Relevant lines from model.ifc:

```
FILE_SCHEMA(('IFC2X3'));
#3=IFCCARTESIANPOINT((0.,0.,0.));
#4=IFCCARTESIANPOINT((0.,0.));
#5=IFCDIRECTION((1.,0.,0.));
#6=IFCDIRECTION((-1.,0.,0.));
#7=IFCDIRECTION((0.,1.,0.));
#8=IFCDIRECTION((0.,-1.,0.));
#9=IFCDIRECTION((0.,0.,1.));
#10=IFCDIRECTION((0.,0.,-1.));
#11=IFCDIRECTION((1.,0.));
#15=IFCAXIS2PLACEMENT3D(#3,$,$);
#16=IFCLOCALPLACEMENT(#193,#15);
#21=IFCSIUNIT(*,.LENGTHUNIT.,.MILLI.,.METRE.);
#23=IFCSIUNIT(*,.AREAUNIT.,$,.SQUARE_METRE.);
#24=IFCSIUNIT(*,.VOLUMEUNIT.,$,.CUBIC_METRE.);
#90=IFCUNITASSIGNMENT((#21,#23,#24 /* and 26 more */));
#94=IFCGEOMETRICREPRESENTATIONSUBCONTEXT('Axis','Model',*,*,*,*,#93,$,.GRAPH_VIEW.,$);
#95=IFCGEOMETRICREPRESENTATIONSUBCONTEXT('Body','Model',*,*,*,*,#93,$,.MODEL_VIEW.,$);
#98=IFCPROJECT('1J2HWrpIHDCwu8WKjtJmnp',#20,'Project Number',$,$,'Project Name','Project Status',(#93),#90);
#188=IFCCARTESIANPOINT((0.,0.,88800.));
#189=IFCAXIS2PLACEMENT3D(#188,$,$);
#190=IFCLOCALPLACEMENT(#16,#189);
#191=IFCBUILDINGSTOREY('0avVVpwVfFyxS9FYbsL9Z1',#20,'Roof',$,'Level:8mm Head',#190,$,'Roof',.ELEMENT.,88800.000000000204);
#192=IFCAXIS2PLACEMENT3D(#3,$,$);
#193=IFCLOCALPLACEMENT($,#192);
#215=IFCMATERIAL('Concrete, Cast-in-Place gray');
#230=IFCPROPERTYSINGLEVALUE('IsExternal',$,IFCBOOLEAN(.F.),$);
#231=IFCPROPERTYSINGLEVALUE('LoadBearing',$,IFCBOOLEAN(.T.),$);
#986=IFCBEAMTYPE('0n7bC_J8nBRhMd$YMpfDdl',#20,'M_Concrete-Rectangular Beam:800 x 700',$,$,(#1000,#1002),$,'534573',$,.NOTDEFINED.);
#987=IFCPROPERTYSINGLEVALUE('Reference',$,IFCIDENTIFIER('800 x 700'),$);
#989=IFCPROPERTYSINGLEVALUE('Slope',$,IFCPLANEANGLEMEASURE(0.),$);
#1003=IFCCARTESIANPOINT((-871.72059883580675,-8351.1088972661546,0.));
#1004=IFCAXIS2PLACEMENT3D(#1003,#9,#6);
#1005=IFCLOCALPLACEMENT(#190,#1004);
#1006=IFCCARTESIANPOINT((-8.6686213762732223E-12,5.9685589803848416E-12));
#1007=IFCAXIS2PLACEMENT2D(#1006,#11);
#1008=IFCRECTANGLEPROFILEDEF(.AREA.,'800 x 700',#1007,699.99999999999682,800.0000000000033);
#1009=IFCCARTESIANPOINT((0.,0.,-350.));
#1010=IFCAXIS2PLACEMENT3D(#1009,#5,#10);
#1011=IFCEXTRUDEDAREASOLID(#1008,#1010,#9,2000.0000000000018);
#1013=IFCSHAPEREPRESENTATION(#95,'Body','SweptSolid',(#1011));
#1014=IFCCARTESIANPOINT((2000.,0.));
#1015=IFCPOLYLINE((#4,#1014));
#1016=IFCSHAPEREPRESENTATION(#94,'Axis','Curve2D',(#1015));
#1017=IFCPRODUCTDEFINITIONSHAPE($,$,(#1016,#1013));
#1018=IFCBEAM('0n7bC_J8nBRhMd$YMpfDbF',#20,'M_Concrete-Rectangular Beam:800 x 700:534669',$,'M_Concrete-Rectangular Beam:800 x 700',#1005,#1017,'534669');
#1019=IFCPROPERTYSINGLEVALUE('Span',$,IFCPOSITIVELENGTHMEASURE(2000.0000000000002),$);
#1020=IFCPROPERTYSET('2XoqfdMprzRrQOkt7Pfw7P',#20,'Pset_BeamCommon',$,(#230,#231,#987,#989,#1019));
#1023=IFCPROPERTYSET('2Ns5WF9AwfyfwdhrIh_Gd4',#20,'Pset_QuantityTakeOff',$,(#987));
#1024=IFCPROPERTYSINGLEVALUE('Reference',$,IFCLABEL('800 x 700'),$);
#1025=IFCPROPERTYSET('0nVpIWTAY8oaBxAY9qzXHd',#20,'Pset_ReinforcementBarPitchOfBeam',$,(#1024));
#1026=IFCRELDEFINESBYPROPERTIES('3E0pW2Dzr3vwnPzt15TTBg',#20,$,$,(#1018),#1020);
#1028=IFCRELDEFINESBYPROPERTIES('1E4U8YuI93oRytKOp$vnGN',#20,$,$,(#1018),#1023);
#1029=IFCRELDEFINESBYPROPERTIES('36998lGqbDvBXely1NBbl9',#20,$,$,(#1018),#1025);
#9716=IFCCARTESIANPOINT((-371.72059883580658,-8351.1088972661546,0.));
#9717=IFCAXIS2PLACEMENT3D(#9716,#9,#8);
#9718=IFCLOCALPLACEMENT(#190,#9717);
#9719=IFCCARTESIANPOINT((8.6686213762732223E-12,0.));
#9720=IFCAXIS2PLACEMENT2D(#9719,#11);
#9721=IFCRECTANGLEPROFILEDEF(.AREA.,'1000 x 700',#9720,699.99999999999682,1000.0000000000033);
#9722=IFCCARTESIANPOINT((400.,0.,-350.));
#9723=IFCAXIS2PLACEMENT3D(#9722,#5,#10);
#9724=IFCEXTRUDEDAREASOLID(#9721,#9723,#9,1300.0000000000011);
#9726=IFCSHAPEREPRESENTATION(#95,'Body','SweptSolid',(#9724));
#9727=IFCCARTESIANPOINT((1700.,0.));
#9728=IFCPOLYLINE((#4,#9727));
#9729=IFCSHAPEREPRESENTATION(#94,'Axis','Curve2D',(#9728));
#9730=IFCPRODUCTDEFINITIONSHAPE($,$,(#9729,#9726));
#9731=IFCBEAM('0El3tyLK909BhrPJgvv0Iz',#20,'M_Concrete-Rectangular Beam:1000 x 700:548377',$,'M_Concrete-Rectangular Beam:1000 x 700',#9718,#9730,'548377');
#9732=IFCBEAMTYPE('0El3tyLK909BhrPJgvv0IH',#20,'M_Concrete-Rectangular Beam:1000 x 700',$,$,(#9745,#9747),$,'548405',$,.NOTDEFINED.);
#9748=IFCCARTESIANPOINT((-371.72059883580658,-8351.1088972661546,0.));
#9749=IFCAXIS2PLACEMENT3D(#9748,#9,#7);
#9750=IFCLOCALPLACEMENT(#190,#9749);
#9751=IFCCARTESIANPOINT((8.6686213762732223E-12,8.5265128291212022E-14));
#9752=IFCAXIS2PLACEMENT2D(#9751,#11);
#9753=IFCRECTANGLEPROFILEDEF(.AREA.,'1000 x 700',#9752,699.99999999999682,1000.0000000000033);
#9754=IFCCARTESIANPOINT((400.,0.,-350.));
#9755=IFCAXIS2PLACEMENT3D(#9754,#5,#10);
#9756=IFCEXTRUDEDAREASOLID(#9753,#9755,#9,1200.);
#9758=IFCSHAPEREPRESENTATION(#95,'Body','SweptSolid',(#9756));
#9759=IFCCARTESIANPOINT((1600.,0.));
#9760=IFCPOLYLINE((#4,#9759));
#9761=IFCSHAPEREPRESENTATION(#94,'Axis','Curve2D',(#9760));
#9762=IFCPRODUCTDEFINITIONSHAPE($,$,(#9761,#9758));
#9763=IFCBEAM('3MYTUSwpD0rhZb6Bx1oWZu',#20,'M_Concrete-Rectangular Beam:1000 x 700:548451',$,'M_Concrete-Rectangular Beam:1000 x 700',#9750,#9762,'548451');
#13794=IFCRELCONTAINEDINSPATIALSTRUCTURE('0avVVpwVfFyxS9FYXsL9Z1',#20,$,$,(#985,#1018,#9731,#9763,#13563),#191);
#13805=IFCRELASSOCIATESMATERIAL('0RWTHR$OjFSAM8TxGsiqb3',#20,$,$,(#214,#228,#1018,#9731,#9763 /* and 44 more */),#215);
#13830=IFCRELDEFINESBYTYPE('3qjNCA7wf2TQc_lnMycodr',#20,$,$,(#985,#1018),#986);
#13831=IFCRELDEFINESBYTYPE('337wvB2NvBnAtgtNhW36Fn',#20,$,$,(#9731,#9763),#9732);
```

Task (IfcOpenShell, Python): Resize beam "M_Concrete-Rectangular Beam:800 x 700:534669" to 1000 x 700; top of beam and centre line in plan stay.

```python
import ifcopenshell
import ifcopenshell.api.pset
import ifcopenshell.api.type
import ifcopenshell.util.element
import ifcopenshell.util.representation

model = ifcopenshell.open("model.ifc")

member = model.by_guid("0n7bC_J8nBRhMd$YMpfDbF")
source = next(p for p in model.by_type("IfcRectangleProfileDef") if p.ProfileName == "1000 x 700")

body = ifcopenshell.util.representation.get_representation(member, "Model", "Body")
solid = body.Items[0]
old_profile = solid.SweptArea

# Copy the section's sizes but keep this member's own profile position.
profile = ifcopenshell.util.element.copy(model, source)
# Profiles are centred, so shift by half the change in depth to hold the top.
shift = (old_profile.XDim - profile.XDim) / 2
x, y = old_profile.Position.Location.Coordinates
up = (-1.0, 0.0)  # upwards, in the solid's own plane
location = model.createIfcCartesianPoint((x + up[0] * shift, y + up[1] * shift))
profile.Position = model.createIfcAxis2Placement2D(location, old_profile.Position.RefDirection)
solid.SweptArea = profile
if not model.get_total_inverses(old_profile):
    ifcopenshell.util.element.remove_deep2(model, old_profile)

new_type = model.by_id(9732)
ifcopenshell.api.type.assign_type(
    model, related_objects=[member], relating_type=new_type, should_map_representations=False
)
member.Name = member.Name.replace("800 x 700", "1000 x 700")
member.ObjectType = "M_Concrete-Rectangular Beam:1000 x 700"
pset = model.by_id(ifcopenshell.util.element.get_pset(member, "Pset_BeamCommon", should_inherit=False)["id"])
ifcopenshell.api.pset.edit_pset(model, pset=pset, properties={"Reference": "1000 x 700"})
pset = model.by_id(ifcopenshell.util.element.get_pset(member, "Pset_QuantityTakeOff", should_inherit=False)["id"])
ifcopenshell.api.pset.edit_pset(model, pset=pset, properties={"Reference": "1000 x 700"})
pset = model.by_id(ifcopenshell.util.element.get_pset(member, "Pset_ReinforcementBarPitchOfBeam", should_inherit=False)["id"])
ifcopenshell.api.pset.edit_pset(model, pset=pset, properties={"Reference": "1000 x 700"})

print(solid.SweptArea)

model.write("model-out.ifc")
```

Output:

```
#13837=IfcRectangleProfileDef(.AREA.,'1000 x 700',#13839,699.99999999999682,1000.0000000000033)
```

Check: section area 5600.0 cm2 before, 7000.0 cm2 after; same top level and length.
